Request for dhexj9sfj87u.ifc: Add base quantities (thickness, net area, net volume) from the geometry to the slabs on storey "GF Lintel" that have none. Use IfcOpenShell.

First a look at what the model holds.

```python
import ifcopenshell
import ifcopenshell.util.element
import ifcopenshell.util.unit

model = ifcopenshell.open("dhexj9sfj87u.ifc")
print(model.schema)
for unit_type in ("LENGTHUNIT", "AREAUNIT", "VOLUMEUNIT"):
    print(unit_type, ifcopenshell.util.unit.calculate_unit_scale(model, unit_type))
storey = next(s for s in model.by_type("IfcBuildingStorey") if s.Name == "GF Lintel")
slabs = [e for e in ifcopenshell.util.element.get_decomposition(storey) if e.is_a("IfcSlab")]
for e in sorted(slabs, key=lambda e: e.id()):
    print(e.id(), e.is_a(), e.Name, list(ifcopenshell.util.element.get_psets(e, qtos_only=True)), sep=" | ")
```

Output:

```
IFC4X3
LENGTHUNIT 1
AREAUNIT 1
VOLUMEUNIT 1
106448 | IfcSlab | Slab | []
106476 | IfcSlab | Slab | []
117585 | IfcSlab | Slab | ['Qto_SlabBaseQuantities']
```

```python
import ifcopenshell
import ifcopenshell.api.pset
import ifcopenshell.geom
import ifcopenshell.util.element
import ifcopenshell.util.shape
import ifcopenshell.util.unit

model = ifcopenshell.open("dhexj9sfj87u.ifc")
unit_scale = ifcopenshell.util.unit.calculate_unit_scale(model)
area_scale = ifcopenshell.util.unit.calculate_unit_scale(model, "AREAUNIT")
volume_scale = ifcopenshell.util.unit.calculate_unit_scale(model, "VOLUMEUNIT")
settings = ifcopenshell.geom.settings()

storey = next(s for s in model.by_type("IfcBuildingStorey") if s.Name == "GF Lintel")
slabs = [e for e in ifcopenshell.util.element.get_decomposition(storey) if e.is_a("IfcSlab")]

for e in sorted(slabs, key=lambda e: e.id()):
    if ifcopenshell.util.element.get_psets(e, qtos_only=True, should_inherit=False):
        continue
    # Geometry comes back in metres, in the element's own axes.
    shape = ifcopenshell.geom.create_shape(settings, e)
    values = {
        "Width": ifcopenshell.util.shape.get_z(shape.geometry) / unit_scale,
        "NetArea": ifcopenshell.util.shape.get_footprint_area(shape.geometry) / area_scale,
        "NetVolume": ifcopenshell.util.shape.get_volume(shape.geometry) / volume_scale,
    }
    qto = ifcopenshell.api.pset.add_qto(model, product=e, name="Qto_SlabBaseQuantities")
    ifcopenshell.api.pset.edit_qto(model, qto=qto, properties=values)
    print(e.id(), {k: round(v, 3) for k, v in values.items()})

model.write("dhexj9sfj87u_updated.ifc")
```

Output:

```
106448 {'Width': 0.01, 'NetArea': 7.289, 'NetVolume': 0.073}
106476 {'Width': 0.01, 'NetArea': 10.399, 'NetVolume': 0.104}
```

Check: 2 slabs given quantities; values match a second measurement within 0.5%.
